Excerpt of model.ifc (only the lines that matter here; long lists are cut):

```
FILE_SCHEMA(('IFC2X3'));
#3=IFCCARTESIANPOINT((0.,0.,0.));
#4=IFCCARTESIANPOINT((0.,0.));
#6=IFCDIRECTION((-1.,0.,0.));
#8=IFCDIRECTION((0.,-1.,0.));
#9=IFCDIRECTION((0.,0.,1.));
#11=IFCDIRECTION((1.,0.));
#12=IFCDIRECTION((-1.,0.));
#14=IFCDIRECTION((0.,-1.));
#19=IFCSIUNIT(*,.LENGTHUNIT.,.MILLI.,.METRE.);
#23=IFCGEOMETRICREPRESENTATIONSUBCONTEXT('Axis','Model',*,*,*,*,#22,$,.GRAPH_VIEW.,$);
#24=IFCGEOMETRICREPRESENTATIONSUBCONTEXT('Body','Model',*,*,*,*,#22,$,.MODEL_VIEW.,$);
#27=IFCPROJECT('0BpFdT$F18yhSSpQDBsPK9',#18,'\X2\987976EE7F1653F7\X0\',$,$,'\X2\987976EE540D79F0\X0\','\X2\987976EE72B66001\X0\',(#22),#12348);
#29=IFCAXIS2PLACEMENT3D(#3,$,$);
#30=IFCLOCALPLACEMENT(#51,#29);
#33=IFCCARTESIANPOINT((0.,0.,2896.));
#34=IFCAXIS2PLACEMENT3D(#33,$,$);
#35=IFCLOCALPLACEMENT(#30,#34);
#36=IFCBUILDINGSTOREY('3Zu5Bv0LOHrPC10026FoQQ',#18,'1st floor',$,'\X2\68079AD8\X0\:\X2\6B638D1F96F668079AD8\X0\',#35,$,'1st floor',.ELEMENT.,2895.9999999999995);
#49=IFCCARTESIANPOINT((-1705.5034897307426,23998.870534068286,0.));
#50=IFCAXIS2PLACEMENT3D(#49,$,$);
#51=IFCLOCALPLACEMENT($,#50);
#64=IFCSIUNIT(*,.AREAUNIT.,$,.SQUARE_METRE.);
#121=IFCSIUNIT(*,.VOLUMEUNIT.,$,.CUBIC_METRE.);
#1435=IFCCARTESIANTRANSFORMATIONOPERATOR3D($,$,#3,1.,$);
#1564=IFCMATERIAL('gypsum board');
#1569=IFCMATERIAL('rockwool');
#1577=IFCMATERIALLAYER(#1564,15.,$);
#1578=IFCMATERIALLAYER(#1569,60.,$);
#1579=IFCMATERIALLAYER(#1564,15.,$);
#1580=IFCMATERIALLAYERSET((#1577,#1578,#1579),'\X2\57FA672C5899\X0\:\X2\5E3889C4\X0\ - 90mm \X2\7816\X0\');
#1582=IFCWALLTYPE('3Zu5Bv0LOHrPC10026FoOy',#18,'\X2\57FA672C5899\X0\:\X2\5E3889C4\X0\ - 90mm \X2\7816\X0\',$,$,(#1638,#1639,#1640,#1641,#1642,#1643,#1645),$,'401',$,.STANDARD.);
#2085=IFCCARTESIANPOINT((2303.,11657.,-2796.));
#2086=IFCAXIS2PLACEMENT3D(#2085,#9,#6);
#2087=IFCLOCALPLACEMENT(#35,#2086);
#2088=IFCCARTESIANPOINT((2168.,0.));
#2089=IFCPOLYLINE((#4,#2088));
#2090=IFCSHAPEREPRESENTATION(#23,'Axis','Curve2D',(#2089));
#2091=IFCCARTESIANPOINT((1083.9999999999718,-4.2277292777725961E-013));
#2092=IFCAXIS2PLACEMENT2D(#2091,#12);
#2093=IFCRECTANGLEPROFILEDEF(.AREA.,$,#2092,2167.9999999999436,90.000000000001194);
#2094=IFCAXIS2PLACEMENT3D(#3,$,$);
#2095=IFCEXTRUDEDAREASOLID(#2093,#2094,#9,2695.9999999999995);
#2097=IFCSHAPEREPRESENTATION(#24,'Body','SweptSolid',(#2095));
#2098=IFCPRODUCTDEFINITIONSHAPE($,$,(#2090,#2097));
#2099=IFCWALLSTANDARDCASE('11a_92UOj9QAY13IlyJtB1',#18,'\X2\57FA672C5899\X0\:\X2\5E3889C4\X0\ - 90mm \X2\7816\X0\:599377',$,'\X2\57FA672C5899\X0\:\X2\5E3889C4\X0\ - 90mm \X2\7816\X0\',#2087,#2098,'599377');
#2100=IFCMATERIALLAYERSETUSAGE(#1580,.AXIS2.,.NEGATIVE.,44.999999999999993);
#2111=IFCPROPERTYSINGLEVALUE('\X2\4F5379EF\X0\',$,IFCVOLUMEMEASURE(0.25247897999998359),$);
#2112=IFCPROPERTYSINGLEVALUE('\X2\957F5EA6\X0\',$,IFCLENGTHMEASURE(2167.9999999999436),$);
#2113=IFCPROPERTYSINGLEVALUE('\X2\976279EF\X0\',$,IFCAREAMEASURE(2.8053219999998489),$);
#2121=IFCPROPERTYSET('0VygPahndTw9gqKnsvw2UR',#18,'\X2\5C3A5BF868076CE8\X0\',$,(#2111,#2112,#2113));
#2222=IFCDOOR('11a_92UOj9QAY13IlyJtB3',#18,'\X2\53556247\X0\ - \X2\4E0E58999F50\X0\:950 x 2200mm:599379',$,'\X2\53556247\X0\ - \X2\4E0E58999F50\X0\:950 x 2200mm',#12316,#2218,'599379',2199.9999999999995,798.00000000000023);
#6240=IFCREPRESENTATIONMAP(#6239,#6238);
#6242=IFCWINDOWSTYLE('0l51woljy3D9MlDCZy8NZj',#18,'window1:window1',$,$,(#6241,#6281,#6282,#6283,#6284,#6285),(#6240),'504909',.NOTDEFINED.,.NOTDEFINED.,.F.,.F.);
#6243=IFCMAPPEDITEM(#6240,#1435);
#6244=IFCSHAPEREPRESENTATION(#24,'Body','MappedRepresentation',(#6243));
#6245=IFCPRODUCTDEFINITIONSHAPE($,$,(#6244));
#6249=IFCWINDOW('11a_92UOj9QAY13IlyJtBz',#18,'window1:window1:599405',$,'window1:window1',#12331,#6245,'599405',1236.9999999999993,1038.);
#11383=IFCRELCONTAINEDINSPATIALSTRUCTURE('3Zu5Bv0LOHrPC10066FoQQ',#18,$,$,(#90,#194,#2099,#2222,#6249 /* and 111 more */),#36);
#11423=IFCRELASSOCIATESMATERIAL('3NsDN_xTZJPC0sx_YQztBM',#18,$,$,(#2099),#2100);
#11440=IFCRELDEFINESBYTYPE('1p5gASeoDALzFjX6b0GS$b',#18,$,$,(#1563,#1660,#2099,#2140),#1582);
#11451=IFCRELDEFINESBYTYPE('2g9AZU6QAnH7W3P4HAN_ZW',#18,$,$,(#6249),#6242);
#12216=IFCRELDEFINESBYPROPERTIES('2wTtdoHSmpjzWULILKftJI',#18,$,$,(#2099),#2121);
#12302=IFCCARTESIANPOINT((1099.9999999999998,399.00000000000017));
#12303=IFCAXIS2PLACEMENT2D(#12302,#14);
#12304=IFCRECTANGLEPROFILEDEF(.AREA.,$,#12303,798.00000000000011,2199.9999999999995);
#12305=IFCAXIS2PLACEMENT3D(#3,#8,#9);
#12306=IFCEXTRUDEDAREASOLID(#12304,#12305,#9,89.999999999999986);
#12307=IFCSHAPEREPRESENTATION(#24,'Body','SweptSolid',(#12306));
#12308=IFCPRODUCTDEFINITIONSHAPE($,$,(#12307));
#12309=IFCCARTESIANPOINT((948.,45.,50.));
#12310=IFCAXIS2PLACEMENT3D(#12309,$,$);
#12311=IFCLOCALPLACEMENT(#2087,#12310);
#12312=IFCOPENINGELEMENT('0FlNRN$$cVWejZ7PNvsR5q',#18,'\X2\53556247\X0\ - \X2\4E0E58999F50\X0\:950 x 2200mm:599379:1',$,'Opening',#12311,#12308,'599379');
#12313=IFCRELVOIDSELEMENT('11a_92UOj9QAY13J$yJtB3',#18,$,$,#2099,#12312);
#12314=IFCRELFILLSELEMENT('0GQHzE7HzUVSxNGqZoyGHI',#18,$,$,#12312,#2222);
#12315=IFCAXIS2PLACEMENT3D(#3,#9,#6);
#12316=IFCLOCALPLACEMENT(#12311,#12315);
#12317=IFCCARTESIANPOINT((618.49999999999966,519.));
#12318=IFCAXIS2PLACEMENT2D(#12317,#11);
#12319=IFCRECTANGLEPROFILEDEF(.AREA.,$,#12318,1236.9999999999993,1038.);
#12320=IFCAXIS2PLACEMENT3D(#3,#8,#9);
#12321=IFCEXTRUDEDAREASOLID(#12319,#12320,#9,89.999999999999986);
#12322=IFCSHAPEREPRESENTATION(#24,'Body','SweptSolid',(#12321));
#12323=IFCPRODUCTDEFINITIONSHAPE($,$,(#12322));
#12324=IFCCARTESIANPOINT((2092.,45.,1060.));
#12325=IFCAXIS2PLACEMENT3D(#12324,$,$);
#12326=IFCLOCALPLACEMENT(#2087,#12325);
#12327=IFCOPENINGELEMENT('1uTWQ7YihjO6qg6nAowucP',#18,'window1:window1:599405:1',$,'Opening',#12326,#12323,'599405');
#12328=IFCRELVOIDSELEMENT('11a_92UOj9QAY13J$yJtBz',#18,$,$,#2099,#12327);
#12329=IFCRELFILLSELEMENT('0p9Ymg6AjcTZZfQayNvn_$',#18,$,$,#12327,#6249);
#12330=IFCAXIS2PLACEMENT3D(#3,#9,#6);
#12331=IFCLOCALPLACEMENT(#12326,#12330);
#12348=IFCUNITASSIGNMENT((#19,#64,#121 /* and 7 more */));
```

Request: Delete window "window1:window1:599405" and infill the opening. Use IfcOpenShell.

```python
import ifcopenshell
import ifcopenshell.api.feature
import ifcopenshell.api.pset
import ifcopenshell.api.root
import ifcopenshell.geom
import ifcopenshell.util.element
import ifcopenshell.util.shape
import ifcopenshell.util.unit

model = ifcopenshell.open("model.ifc")
area_scale = ifcopenshell.util.unit.calculate_unit_scale(model, "AREAUNIT")
volume_scale = ifcopenshell.util.unit.calculate_unit_scale(model, "VOLUMEUNIT")
settings = ifcopenshell.geom.settings()


def volume(element):
    """Net volume in cubic metres, openings subtracted."""
    shape = ifcopenshell.geom.create_shape(settings, element)
    return ifcopenshell.util.shape.get_volume(shape.geometry)


window = model.by_id(6249)
opening = window.FillsVoids[0].RelatingOpeningElement
wall = opening.VoidsElements[0].RelatingBuildingElement
before = volume(wall)

ifcopenshell.api.root.remove_product(model, product=window)
ifcopenshell.api.feature.remove_feature(model, feature=opening)

after = volume(wall)
thickness = 0.09  # wall thickness in metres

# Update the wall's stored quantities.
pset = model.by_id(ifcopenshell.util.element.get_pset(wall, "尺寸标注", should_inherit=False)["id"])
ifcopenshell.api.pset.edit_pset(model, pset=pset, properties={
    "体积": model.create_entity("IfcVolumeMeasure", after / volume_scale),
    "面积": model.create_entity("IfcAreaMeasure", after / thickness / area_scale),
})

print(f"wall volume {before:.3f} -> {after:.3f} m3")

model.write("model_rev.ifc")
```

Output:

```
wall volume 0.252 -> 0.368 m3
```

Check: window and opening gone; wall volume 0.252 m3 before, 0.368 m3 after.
